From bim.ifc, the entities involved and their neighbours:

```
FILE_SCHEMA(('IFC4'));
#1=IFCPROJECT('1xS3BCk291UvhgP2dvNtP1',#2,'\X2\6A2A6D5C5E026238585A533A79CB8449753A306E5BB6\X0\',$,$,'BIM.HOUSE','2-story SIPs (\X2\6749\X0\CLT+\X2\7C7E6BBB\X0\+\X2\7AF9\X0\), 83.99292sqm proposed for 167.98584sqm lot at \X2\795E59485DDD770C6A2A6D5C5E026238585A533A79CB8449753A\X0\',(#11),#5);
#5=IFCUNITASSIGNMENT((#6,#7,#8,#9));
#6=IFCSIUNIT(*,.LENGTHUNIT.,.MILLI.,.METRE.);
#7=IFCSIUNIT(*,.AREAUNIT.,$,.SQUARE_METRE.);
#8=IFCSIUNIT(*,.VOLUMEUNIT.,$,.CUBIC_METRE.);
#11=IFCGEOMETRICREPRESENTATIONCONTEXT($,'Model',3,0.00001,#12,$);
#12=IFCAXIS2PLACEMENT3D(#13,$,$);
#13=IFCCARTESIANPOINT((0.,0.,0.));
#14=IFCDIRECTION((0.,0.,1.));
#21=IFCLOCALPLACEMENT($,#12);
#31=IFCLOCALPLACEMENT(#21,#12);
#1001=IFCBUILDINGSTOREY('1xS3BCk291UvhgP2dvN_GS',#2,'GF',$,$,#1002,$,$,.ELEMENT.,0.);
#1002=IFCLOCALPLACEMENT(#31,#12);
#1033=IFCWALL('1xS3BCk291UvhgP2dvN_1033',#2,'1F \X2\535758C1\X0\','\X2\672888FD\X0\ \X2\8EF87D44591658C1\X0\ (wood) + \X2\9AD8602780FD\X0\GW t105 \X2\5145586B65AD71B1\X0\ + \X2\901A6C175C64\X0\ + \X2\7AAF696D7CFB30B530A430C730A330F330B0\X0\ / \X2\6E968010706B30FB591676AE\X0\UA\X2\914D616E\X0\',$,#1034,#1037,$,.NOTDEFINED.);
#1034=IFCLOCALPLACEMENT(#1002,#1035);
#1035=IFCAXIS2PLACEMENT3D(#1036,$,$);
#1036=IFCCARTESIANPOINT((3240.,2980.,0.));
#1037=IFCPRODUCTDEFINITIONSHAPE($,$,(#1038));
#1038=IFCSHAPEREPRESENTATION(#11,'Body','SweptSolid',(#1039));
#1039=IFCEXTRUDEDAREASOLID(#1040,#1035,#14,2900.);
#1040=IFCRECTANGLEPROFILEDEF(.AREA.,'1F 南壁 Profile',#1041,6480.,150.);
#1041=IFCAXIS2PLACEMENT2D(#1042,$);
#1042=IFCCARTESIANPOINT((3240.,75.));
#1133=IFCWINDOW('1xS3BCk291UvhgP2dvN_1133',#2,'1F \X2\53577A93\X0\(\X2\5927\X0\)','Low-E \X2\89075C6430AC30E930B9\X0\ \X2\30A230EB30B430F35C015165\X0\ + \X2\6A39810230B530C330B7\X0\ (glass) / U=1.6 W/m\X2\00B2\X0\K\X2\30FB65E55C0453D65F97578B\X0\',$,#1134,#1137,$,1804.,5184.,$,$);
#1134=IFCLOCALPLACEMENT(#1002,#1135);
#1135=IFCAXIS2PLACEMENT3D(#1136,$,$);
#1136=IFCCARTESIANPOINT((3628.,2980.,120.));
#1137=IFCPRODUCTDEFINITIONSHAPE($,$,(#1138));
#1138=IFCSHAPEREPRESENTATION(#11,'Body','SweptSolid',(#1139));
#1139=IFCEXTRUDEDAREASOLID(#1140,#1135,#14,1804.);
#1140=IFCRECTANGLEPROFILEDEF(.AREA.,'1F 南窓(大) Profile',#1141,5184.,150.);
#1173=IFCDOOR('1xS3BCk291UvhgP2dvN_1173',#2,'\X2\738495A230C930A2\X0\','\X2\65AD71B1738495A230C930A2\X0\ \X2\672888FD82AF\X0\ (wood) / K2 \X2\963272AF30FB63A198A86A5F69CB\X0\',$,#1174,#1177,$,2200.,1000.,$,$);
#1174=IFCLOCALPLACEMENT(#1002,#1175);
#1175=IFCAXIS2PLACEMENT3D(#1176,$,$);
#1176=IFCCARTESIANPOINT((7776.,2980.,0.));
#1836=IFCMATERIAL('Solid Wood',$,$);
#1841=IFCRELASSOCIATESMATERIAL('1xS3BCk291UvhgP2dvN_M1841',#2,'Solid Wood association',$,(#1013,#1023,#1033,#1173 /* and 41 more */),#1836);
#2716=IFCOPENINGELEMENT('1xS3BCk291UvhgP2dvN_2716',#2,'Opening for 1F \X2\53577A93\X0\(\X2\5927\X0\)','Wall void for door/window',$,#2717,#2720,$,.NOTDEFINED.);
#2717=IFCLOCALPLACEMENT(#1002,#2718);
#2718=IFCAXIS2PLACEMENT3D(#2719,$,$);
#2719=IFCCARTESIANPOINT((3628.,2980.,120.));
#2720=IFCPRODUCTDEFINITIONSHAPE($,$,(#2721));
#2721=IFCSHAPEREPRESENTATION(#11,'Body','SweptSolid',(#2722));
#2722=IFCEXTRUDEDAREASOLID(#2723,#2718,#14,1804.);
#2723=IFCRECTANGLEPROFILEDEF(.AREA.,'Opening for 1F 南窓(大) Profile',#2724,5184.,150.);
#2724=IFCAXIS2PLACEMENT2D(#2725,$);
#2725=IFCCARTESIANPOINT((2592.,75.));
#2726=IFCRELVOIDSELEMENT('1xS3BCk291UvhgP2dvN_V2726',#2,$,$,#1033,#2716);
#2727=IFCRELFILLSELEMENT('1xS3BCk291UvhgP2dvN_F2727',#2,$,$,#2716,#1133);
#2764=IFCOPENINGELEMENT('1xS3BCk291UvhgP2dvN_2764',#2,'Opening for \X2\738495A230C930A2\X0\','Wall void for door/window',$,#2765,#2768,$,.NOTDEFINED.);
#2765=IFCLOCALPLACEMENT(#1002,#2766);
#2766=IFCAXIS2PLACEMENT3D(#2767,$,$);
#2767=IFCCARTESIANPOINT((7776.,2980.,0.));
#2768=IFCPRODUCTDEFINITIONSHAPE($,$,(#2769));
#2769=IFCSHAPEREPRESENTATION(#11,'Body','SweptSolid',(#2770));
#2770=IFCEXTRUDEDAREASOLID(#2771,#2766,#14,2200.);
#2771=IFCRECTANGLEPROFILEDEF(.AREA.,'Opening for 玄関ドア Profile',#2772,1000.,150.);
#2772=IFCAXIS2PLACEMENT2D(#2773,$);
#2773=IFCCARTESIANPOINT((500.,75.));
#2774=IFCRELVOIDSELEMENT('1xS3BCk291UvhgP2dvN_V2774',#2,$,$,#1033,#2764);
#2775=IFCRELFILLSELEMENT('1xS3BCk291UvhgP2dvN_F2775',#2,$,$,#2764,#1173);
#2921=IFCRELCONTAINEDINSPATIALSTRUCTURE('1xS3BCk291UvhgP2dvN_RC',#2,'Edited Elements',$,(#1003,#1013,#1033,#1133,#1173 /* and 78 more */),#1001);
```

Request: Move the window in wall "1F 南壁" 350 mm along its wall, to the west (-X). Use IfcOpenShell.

```python
import ifcopenshell
import ifcopenshell.api.geometry
import ifcopenshell.util.placement

model = ifcopenshell.open("bim.ifc")

window = model.by_guid("1xS3BCk291UvhgP2dvN_1133")
opening = window.FillsVoids[0].RelatingOpeningElement
wall = opening.VoidsElements[0].RelatingBuildingElement

wall_matrix = ifcopenshell.util.placement.get_local_placement(wall.ObjectPlacement)
shift = wall_matrix[:3, 0] * -350.0
before = ifcopenshell.util.placement.get_local_placement(window.ObjectPlacement)[:3, 3].copy()

# The window is not placed relative to its opening, so move both.
for product in (opening, window):
    matrix = ifcopenshell.util.placement.get_local_placement(product.ObjectPlacement)
    matrix[:3, 3] += shift
    ifcopenshell.api.geometry.edit_object_placement(model, product=product, matrix=matrix, is_si=False)

after = ifcopenshell.util.placement.get_local_placement(window.ObjectPlacement)[:3, 3]
print("window moved by", (after - before).round(3) + 0.0)

model.write("bim-out.ifc")
```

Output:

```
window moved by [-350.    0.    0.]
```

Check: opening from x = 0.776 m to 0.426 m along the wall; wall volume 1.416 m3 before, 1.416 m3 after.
